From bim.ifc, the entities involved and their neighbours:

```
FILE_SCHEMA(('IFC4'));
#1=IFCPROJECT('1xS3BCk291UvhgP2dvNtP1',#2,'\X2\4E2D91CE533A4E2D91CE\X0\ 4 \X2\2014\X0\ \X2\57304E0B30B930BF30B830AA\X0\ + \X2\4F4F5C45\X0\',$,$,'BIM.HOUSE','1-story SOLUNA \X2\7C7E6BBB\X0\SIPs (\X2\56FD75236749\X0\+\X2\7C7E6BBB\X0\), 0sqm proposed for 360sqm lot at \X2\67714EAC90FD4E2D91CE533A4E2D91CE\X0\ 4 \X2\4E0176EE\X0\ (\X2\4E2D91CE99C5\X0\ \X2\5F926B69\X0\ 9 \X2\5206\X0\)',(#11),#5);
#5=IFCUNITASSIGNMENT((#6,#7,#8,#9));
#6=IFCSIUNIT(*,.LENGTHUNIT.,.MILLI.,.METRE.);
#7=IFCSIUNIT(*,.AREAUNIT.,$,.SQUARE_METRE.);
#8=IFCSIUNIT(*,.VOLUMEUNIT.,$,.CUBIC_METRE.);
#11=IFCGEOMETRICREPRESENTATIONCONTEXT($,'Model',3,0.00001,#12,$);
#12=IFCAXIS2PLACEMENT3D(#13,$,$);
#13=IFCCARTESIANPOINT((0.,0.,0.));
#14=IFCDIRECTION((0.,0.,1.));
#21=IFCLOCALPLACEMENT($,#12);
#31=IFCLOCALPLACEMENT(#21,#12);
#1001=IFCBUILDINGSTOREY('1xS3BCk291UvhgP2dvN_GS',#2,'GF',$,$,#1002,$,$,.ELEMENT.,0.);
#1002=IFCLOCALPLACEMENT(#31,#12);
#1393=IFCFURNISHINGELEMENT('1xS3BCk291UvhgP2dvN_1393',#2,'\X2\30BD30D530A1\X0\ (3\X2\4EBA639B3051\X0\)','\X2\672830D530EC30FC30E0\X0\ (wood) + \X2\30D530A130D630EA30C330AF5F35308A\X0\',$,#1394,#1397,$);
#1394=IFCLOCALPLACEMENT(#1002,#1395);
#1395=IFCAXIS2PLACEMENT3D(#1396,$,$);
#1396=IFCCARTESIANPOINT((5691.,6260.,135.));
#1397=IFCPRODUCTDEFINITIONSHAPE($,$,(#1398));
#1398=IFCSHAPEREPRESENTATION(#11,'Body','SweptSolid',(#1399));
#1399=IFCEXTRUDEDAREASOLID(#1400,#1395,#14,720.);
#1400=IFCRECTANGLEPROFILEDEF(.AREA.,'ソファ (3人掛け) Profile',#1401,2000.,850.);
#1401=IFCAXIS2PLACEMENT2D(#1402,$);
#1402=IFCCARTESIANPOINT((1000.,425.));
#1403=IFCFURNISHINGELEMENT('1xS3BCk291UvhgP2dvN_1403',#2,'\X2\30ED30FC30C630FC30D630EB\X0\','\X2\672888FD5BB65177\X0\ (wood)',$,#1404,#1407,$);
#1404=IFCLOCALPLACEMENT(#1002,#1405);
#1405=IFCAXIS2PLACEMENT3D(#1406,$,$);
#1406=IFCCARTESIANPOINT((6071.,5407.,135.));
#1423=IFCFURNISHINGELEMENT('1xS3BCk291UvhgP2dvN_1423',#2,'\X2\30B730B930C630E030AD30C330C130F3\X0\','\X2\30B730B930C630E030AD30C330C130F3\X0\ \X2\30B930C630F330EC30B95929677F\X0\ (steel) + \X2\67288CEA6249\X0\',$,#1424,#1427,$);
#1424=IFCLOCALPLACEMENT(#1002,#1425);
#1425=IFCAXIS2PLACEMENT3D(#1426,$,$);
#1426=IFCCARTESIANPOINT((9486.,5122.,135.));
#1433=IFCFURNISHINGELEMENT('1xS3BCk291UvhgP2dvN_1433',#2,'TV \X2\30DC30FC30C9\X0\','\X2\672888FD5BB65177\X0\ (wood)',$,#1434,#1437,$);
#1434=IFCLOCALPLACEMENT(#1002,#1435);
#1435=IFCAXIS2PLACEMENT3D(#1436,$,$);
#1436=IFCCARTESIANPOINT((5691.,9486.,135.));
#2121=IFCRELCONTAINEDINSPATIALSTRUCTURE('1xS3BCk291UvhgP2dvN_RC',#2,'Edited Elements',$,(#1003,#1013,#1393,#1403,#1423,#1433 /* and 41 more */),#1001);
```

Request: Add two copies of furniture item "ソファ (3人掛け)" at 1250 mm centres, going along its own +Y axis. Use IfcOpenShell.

```python
import ifcopenshell
import ifcopenshell.api.geometry
import ifcopenshell.api.root
import ifcopenshell.util.element
import ifcopenshell.util.placement
import ifcopenshell.util.unit

model = ifcopenshell.open("bim.ifc")
unit_scale = ifcopenshell.util.unit.calculate_unit_scale(model)


def reuse_history(source, copy):
    """copy_class also copies each property set's owner history, people and application; keep the originals."""
    for rel in copy.IsDefinedBy:
        if rel.is_a("IfcRelDefinesByProperties") and (history := rel.RelatingPropertyDefinition.OwnerHistory):
            rel.RelatingPropertyDefinition.OwnerHistory = source.OwnerHistory
            ifcopenshell.util.element.remove_deep2(model, history)


source = model.by_id(1393)
base = ifcopenshell.util.placement.get_local_placement(source.ObjectPlacement)
step = base[:3, 1] * 1.25 / unit_scale

for i in range(1, 3):
    copy = ifcopenshell.api.root.copy_class(model, product=source)
    copy.Representation = ifcopenshell.util.element.copy_deep(
        model, source.Representation, exclude=["IfcGeometricRepresentationContext", "IfcRepresentationMap"]
    )
    reuse_history(source, copy)
    matrix = base.copy()
    matrix[:3, 3] += i * step
    print("added at", matrix[:3, 3].round(3) + 0.0)
    ifcopenshell.api.geometry.edit_object_placement(model, product=copy, matrix=matrix, is_si=False)

model.write("bim_rev.ifc")
```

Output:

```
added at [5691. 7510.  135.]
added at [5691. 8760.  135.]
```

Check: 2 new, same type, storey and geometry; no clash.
